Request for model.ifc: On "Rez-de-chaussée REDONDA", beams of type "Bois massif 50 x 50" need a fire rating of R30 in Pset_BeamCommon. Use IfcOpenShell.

First a look at what the model holds.

```python
import ifcopenshell
import ifcopenshell.util.element

model = ifcopenshell.open("model.ifc")
print(model.schema)
storey = next(s for s in model.by_type("IfcBuildingStorey") if s.Name == "Rez-de-chaussée REDONDA")
beams = [e for e in ifcopenshell.util.element.get_decomposition(storey) if e.is_a("IfcBeam")]
seen = {}
for e in beams:
    element_type = ifcopenshell.util.element.get_type(e)
    key = (element_type.Name if element_type != e and element_type else None, ifcopenshell.util.element.get_pset(e, "Pset_BeamCommon", "FireRating"))
    seen[key] = seen.get(key, 0) + 1
for (name, value), count in sorted(seen.items(), key=str):
    print(count, "x", name, "|", value)
```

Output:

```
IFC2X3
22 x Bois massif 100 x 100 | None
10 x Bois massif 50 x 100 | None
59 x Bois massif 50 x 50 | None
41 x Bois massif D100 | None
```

```python
import ifcopenshell
import ifcopenshell.api.pset
import ifcopenshell.util.element

model = ifcopenshell.open("model.ifc")

storey = next(s for s in model.by_type("IfcBuildingStorey") if s.Name == "Rez-de-chaussée REDONDA")
beams = [e for e in ifcopenshell.util.element.get_decomposition(storey) if e.is_a("IfcBeam")]

count = 0
for e in beams:
    element_type = ifcopenshell.util.element.get_type(e)
    if element_type in (None, e) or element_type.Name != "Bois massif 50 x 50":
        continue
    # add_pset returns the element's existing set when there is one.
    pset = ifcopenshell.api.pset.add_pset(model, product=e, name="Pset_BeamCommon")
    ifcopenshell.api.pset.edit_pset(model, pset=pset, properties={"FireRating": "R30"})
    count += 1

print(count, "beams updated")

model.write("model_rev.ifc")
```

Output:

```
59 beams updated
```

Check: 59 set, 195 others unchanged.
